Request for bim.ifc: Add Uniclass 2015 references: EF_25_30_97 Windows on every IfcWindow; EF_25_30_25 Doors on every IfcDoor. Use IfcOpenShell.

First a look at what the model holds.

```python
import ifcopenshell

model = ifcopenshell.open("bim.ifc")
print(model.schema)
print("classifications:", [c.Name for c in model.by_type("IfcClassification")])
for ifc_class in ("IfcDoor", "IfcRoof", "IfcStair", "IfcWall", "IfcWindow"):
    print(ifc_class, len(model.by_type(ifc_class)))
```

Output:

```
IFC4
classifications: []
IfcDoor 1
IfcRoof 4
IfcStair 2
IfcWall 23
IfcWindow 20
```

```python
import ifcopenshell
import ifcopenshell.api.classification

model = ifcopenshell.open("bim.ifc")

system = ifcopenshell.api.classification.add_classification(model, classification="Uniclass 2015")

codes = {
    "IfcWindow": ("EF_25_30_97", "Windows"),
    "IfcDoor": ("EF_25_30_25", "Doors"),
}
for ifc_class, (code, name) in codes.items():
    products = model.by_type(ifc_class)
    ifcopenshell.api.classification.add_reference(
        model, products=products, classification=system, identification=code, name=name
    )
    print(code, len(products))

model.write("bim_rev.ifc")
```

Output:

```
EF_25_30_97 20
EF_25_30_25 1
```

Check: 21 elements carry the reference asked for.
